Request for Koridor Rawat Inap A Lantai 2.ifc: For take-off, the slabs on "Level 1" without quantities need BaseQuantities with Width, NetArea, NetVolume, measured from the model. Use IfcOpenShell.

First a look at what the model holds.

```python
import ifcopenshell
import ifcopenshell.util.element
import ifcopenshell.util.unit

model = ifcopenshell.open("Koridor Rawat Inap A Lantai 2.ifc")
print(model.schema)
for unit_type in ("LENGTHUNIT", "AREAUNIT", "VOLUMEUNIT"):
    print(unit_type, ifcopenshell.util.unit.calculate_unit_scale(model, unit_type))
storey = next(s for s in model.by_type("IfcBuildingStorey") if s.Name == "Level 1")
slabs = [e for e in ifcopenshell.util.element.get_decomposition(storey) if e.is_a("IfcSlab")]
for e in sorted(slabs, key=lambda e: e.id()):
    print(e.id(), e.is_a(), e.Name, list(ifcopenshell.util.element.get_psets(e, qtos_only=True)), sep=" | ")
```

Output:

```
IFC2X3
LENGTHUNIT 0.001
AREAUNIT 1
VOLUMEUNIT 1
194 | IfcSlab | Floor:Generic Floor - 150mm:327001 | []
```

```python
import ifcopenshell
import ifcopenshell.api.pset
import ifcopenshell.geom
import ifcopenshell.util.element
import ifcopenshell.util.shape
import ifcopenshell.util.unit

model = ifcopenshell.open("Koridor Rawat Inap A Lantai 2.ifc")
unit_scale = ifcopenshell.util.unit.calculate_unit_scale(model)
area_scale = ifcopenshell.util.unit.calculate_unit_scale(model, "AREAUNIT")
volume_scale = ifcopenshell.util.unit.calculate_unit_scale(model, "VOLUMEUNIT")
settings = ifcopenshell.geom.settings()

storey = next(s for s in model.by_type("IfcBuildingStorey") if s.Name == "Level 1")
slabs = [e for e in ifcopenshell.util.element.get_decomposition(storey) if e.is_a("IfcSlab")]

for e in sorted(slabs, key=lambda e: e.id()):
    if ifcopenshell.util.element.get_psets(e, qtos_only=True, should_inherit=False):
        continue
    # Geometry comes back in metres, in the element's own axes.
    shape = ifcopenshell.geom.create_shape(settings, e)
    values = {
        "Width": ifcopenshell.util.shape.get_z(shape.geometry) / unit_scale,
        "NetArea": ifcopenshell.util.shape.get_footprint_area(shape.geometry) / area_scale,
        "NetVolume": ifcopenshell.util.shape.get_volume(shape.geometry) / volume_scale,
    }
    qto = ifcopenshell.api.pset.add_qto(model, product=e, name="BaseQuantities")
    ifcopenshell.api.pset.edit_qto(model, qto=qto, properties=values)
    print(e.id(), {k: round(v, 3) for k, v in values.items()})

model.write("Koridor Rawat Inap A Lantai 2_v2.ifc")
```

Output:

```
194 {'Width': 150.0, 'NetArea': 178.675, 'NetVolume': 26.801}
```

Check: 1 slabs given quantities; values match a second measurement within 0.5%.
